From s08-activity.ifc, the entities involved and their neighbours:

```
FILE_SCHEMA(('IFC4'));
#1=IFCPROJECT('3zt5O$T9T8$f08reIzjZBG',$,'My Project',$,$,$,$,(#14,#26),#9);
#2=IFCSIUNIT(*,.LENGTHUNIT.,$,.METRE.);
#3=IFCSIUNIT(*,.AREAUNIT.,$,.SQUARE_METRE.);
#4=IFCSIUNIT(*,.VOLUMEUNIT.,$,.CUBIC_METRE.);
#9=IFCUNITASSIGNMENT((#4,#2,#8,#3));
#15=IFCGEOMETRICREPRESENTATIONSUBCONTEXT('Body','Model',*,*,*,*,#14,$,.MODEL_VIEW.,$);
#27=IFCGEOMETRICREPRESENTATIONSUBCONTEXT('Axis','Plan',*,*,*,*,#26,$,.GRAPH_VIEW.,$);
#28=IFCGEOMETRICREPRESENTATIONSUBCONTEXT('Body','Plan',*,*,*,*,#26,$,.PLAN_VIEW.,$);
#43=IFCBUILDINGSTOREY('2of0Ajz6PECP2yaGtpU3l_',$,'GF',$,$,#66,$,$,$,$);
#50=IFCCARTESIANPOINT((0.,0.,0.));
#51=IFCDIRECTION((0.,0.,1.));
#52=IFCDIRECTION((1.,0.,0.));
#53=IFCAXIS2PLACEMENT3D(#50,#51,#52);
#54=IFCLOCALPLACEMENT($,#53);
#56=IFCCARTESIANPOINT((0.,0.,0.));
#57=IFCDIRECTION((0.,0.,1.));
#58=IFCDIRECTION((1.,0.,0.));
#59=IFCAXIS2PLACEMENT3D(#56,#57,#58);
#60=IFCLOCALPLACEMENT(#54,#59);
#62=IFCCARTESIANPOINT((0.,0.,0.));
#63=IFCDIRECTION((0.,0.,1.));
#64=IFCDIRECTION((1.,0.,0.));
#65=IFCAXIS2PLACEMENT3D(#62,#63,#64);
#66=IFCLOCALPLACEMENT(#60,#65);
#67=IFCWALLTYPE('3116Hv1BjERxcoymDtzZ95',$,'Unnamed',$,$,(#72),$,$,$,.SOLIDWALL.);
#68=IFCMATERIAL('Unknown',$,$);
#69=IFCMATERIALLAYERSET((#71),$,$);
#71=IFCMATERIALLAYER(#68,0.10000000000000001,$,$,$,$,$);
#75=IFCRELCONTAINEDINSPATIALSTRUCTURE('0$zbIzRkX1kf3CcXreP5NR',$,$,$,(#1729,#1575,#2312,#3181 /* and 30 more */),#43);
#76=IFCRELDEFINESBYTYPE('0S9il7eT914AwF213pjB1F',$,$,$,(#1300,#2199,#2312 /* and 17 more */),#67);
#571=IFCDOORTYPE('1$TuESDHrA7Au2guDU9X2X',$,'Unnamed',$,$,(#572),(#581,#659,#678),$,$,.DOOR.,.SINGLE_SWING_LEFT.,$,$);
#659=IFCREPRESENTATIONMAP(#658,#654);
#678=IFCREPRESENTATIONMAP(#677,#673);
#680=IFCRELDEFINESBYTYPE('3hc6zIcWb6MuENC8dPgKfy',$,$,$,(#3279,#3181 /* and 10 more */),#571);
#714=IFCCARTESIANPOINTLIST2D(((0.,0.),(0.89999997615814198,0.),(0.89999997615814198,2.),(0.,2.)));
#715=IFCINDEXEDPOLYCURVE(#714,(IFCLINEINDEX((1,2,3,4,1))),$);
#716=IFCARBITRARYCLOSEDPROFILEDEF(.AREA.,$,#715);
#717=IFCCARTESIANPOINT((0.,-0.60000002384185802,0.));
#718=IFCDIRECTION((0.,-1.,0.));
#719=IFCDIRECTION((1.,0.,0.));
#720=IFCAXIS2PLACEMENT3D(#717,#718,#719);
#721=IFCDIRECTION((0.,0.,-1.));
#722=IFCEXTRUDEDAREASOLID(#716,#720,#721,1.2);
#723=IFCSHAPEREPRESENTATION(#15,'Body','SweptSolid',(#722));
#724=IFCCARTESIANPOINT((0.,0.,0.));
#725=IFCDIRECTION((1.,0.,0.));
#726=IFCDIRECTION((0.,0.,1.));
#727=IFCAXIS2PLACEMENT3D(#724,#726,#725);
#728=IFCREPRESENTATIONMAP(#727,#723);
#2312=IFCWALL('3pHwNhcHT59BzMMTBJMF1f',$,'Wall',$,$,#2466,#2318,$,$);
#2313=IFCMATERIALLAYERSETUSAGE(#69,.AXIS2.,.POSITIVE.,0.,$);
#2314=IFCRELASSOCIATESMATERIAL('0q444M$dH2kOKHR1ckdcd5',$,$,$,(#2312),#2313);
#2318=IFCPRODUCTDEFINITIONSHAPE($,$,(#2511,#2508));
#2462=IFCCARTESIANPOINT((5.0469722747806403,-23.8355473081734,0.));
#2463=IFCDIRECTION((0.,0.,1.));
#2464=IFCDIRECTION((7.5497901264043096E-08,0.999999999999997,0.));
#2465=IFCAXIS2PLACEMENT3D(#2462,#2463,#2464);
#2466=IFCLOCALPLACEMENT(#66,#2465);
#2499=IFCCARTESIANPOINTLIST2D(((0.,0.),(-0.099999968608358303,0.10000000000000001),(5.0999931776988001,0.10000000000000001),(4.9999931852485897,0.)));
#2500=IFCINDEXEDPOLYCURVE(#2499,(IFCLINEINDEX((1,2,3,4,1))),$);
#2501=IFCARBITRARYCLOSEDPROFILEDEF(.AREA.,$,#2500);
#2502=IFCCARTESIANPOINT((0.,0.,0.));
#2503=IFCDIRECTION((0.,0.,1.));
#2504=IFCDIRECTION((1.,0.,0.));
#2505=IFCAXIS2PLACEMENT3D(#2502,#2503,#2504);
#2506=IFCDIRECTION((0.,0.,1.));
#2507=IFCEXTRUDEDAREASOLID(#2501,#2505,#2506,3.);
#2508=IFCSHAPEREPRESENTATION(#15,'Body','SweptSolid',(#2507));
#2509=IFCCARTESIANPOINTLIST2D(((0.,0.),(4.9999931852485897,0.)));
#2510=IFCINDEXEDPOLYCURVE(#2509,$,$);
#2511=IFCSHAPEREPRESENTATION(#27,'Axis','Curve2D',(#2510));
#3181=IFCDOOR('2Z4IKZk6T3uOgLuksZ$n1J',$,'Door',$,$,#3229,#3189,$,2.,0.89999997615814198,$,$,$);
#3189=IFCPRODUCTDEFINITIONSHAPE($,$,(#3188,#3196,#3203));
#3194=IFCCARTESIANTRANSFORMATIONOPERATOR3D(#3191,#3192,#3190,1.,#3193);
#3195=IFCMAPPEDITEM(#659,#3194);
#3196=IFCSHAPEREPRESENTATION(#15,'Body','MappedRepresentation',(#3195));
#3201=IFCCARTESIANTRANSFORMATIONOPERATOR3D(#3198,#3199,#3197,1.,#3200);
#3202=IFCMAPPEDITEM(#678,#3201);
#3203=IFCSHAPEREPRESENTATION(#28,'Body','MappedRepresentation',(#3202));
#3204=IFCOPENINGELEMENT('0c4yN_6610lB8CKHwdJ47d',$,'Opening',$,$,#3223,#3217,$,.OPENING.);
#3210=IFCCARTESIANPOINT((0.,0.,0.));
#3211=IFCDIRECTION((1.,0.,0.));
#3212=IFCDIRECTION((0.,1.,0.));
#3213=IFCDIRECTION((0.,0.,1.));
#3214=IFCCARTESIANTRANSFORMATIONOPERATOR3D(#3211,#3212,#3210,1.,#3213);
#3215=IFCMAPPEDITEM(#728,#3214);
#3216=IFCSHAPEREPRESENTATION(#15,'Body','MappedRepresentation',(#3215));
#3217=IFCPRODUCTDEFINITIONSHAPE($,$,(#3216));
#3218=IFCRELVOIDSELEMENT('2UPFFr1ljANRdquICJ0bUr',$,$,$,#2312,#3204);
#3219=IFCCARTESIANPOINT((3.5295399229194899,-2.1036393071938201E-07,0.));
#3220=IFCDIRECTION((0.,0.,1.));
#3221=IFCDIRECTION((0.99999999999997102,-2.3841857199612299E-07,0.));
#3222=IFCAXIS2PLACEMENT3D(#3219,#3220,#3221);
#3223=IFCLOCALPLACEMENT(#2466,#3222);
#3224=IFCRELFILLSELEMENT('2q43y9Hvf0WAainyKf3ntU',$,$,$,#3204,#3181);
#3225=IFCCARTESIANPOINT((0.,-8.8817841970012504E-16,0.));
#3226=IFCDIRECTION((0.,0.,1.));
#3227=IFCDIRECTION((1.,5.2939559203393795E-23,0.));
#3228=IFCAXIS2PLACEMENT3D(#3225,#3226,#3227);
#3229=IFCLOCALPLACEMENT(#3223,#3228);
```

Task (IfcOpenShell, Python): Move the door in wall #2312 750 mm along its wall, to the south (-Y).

```python
import ifcopenshell
import ifcopenshell.api.geometry
import ifcopenshell.util.placement

model = ifcopenshell.open("s08-activity.ifc")

door = model.by_guid("2Z4IKZk6T3uOgLuksZ$n1J")
opening = door.FillsVoids[0].RelatingOpeningElement
wall = opening.VoidsElements[0].RelatingBuildingElement

wall_matrix = ifcopenshell.util.placement.get_local_placement(wall.ObjectPlacement)
shift = wall_matrix[:3, 0] * -0.75
before = ifcopenshell.util.placement.get_local_placement(door.ObjectPlacement)[:3, 3].copy()

# The door is placed relative to its opening, so it follows when the opening moves.
matrix = ifcopenshell.util.placement.get_local_placement(opening.ObjectPlacement)
matrix[:3, 3] += shift
ifcopenshell.api.geometry.edit_object_placement(
    model, product=opening, matrix=matrix, is_si=False, should_transform_children=True
)

after = ifcopenshell.util.placement.get_local_placement(door.ObjectPlacement)[:3, 3]
print("door moved by", (after - before).round(3) + 0.0)

model.write("s08-activity_rev.ifc")
```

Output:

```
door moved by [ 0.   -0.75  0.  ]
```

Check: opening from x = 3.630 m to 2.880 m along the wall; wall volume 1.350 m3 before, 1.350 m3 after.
